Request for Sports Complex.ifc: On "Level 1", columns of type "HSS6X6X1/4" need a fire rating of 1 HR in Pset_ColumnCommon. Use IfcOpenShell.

First a look at what the model holds.

```python
import ifcopenshell
import ifcopenshell.util.element

model = ifcopenshell.open("Sports Complex.ifc")
print(model.schema)
storey = next(s for s in model.by_type("IfcBuildingStorey") if s.Name == "Level 1")
columns = [e for e in ifcopenshell.util.element.get_decomposition(storey) if e.is_a("IfcColumn")]
seen = {}
for e in columns:
    element_type = ifcopenshell.util.element.get_type(e)
    key = (element_type.Name if element_type != e and element_type else None, ifcopenshell.util.element.get_pset(e, "Pset_ColumnCommon", "FireRating"))
    seen[key] = seen.get(key, 0) + 1
for (name, value), count in sorted(seen.items(), key=str):
    print(count, "x", name, "|", value)
```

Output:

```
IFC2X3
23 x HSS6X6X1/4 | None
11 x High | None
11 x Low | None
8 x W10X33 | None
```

```python
import ifcopenshell
import ifcopenshell.api.pset
import ifcopenshell.util.element

model = ifcopenshell.open("Sports Complex.ifc")

storey = next(s for s in model.by_type("IfcBuildingStorey") if s.Name == "Level 1")
columns = [e for e in ifcopenshell.util.element.get_decomposition(storey) if e.is_a("IfcColumn")]

count = 0
for e in columns:
    element_type = ifcopenshell.util.element.get_type(e)
    if element_type in (None, e) or element_type.Name != "HSS6X6X1/4":
        continue
    # add_pset returns the element's existing set when there is one.
    pset = ifcopenshell.api.pset.add_pset(model, product=e, name="Pset_ColumnCommon")
    ifcopenshell.api.pset.edit_pset(model, pset=pset, properties={"FireRating": "1 HR"})
    count += 1

print(count, "columns updated")

model.write("Sports Complex_rev.ifc")
```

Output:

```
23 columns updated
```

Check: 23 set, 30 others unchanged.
